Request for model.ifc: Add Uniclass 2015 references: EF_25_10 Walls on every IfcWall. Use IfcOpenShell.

First a look at what the model holds.

```python
import ifcopenshell

model = ifcopenshell.open("model.ifc")
print(model.schema)
print("classifications:", [c.Name for c in model.by_type("IfcClassification")])
for ifc_class in ("IfcDoor", "IfcRoof", "IfcStair", "IfcWall", "IfcWindow"):
    print(ifc_class, len(model.by_type(ifc_class)))
```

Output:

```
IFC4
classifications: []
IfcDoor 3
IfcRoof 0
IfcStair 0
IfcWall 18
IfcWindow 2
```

```python
import ifcopenshell
import ifcopenshell.api.classification

model = ifcopenshell.open("model.ifc")

system = ifcopenshell.api.classification.add_classification(model, classification="Uniclass 2015")

codes = {
    "IfcWall": ("EF_25_10", "Walls"),
}
for ifc_class, (code, name) in codes.items():
    products = model.by_type(ifc_class)
    ifcopenshell.api.classification.add_reference(
        model, products=products, classification=system, identification=code, name=name
    )
    print(code, len(products))

model.write("model-out.ifc")
```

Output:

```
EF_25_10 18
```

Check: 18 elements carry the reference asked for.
